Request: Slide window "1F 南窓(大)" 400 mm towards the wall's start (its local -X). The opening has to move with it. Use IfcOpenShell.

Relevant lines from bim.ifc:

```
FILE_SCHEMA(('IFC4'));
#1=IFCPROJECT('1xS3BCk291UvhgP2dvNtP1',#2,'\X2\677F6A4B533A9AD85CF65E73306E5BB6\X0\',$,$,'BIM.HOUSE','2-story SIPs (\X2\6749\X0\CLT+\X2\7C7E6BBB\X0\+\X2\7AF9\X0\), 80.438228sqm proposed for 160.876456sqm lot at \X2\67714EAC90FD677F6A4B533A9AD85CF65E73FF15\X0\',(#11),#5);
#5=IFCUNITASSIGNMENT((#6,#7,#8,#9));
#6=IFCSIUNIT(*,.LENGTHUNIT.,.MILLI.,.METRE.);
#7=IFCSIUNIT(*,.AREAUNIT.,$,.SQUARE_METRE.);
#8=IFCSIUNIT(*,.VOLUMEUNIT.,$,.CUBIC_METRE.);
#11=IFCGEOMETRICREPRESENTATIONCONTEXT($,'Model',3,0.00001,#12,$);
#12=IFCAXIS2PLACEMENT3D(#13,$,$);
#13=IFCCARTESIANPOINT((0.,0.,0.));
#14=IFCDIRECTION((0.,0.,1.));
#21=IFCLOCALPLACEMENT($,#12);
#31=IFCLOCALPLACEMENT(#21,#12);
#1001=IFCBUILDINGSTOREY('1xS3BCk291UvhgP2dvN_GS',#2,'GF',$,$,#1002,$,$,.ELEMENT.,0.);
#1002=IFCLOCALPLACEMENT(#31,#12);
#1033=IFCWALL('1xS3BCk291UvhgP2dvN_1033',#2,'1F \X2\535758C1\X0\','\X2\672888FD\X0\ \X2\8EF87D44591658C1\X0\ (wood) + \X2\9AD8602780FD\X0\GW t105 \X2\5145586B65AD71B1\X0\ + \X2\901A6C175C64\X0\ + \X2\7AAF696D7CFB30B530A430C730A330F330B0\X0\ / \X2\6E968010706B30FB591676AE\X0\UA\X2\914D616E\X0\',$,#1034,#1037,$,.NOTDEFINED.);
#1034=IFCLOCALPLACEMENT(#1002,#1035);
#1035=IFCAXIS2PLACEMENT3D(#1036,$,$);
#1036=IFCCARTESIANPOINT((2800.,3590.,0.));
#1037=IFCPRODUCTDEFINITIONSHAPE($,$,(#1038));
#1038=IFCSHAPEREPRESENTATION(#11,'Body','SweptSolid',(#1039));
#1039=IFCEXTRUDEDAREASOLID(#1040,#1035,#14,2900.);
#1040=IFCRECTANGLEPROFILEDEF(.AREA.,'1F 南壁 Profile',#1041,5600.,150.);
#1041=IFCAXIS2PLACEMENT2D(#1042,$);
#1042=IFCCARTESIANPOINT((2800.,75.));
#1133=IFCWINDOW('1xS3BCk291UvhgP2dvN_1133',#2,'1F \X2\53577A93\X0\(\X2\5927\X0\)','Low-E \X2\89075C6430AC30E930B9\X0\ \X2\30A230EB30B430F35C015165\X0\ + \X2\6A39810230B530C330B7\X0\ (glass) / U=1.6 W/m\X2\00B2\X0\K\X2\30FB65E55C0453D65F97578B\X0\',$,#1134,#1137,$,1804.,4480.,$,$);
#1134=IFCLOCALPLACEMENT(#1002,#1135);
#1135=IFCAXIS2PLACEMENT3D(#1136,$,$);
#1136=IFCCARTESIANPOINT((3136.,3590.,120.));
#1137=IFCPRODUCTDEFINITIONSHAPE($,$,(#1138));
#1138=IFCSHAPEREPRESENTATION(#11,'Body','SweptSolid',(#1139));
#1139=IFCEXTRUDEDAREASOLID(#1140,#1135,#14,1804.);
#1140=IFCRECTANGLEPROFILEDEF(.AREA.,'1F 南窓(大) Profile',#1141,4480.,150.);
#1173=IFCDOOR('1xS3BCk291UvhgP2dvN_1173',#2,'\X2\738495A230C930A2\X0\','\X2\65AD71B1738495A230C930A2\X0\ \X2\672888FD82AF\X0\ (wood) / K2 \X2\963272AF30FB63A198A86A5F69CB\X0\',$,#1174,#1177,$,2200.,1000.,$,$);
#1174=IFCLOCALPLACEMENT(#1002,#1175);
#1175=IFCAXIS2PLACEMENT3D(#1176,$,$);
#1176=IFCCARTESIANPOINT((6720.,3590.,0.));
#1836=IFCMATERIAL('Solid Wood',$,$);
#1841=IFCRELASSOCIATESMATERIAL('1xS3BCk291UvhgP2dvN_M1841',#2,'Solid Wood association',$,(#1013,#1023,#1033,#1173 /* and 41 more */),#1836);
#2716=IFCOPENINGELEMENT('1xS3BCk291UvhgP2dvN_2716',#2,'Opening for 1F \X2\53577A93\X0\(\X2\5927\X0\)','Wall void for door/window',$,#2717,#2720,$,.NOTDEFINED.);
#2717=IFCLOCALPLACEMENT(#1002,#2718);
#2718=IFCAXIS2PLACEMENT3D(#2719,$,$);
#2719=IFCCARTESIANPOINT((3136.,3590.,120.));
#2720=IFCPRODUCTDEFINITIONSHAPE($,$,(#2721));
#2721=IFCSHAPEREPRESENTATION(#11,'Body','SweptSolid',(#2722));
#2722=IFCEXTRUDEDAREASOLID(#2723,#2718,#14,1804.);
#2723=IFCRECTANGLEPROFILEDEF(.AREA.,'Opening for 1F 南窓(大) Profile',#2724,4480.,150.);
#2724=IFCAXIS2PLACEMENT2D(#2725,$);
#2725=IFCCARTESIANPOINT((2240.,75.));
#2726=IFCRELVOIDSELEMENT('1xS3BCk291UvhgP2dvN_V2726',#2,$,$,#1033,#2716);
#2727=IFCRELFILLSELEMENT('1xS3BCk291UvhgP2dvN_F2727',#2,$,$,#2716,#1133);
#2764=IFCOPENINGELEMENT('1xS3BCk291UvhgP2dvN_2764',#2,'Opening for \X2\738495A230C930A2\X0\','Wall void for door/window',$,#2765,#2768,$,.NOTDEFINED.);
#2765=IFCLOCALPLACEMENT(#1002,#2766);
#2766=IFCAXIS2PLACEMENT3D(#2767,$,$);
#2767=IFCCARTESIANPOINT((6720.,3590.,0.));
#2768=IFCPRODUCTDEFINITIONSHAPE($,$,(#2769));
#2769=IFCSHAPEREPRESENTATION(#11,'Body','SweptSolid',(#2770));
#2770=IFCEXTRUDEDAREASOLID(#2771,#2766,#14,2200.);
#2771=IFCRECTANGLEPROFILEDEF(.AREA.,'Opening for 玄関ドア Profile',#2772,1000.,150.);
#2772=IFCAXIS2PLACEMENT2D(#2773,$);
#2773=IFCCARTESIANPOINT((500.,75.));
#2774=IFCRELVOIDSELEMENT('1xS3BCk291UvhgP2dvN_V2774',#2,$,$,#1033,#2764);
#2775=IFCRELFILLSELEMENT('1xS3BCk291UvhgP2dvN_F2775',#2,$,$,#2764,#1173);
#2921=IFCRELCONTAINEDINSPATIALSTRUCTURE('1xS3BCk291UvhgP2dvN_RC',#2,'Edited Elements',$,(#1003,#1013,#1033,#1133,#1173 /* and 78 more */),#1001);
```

```python
import ifcopenshell
import ifcopenshell.api.geometry
import ifcopenshell.util.placement
import ifcopenshell.util.unit

model = ifcopenshell.open("bim.ifc")
unit_scale = ifcopenshell.util.unit.calculate_unit_scale(model)

window = model.by_guid("1xS3BCk291UvhgP2dvN_1133")
opening = window.FillsVoids[0].RelatingOpeningElement
wall = opening.VoidsElements[0].RelatingBuildingElement

wall_matrix = ifcopenshell.util.placement.get_local_placement(wall.ObjectPlacement)
shift = wall_matrix[:3, 0] * -0.4 / unit_scale
before = ifcopenshell.util.placement.get_local_placement(window.ObjectPlacement)[:3, 3].copy()

# The window is not placed relative to its opening, so move both.
for product in (opening, window):
    matrix = ifcopenshell.util.placement.get_local_placement(product.ObjectPlacement)
    matrix[:3, 3] += shift
    ifcopenshell.api.geometry.edit_object_placement(model, product=product, matrix=matrix, is_si=False)

after = ifcopenshell.util.placement.get_local_placement(window.ObjectPlacement)[:3, 3]
print("window moved by", (after - before).round(3) + 0.0)

model.write("bim_edited.ifc")
```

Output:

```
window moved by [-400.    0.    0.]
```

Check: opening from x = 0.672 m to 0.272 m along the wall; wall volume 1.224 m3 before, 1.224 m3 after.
